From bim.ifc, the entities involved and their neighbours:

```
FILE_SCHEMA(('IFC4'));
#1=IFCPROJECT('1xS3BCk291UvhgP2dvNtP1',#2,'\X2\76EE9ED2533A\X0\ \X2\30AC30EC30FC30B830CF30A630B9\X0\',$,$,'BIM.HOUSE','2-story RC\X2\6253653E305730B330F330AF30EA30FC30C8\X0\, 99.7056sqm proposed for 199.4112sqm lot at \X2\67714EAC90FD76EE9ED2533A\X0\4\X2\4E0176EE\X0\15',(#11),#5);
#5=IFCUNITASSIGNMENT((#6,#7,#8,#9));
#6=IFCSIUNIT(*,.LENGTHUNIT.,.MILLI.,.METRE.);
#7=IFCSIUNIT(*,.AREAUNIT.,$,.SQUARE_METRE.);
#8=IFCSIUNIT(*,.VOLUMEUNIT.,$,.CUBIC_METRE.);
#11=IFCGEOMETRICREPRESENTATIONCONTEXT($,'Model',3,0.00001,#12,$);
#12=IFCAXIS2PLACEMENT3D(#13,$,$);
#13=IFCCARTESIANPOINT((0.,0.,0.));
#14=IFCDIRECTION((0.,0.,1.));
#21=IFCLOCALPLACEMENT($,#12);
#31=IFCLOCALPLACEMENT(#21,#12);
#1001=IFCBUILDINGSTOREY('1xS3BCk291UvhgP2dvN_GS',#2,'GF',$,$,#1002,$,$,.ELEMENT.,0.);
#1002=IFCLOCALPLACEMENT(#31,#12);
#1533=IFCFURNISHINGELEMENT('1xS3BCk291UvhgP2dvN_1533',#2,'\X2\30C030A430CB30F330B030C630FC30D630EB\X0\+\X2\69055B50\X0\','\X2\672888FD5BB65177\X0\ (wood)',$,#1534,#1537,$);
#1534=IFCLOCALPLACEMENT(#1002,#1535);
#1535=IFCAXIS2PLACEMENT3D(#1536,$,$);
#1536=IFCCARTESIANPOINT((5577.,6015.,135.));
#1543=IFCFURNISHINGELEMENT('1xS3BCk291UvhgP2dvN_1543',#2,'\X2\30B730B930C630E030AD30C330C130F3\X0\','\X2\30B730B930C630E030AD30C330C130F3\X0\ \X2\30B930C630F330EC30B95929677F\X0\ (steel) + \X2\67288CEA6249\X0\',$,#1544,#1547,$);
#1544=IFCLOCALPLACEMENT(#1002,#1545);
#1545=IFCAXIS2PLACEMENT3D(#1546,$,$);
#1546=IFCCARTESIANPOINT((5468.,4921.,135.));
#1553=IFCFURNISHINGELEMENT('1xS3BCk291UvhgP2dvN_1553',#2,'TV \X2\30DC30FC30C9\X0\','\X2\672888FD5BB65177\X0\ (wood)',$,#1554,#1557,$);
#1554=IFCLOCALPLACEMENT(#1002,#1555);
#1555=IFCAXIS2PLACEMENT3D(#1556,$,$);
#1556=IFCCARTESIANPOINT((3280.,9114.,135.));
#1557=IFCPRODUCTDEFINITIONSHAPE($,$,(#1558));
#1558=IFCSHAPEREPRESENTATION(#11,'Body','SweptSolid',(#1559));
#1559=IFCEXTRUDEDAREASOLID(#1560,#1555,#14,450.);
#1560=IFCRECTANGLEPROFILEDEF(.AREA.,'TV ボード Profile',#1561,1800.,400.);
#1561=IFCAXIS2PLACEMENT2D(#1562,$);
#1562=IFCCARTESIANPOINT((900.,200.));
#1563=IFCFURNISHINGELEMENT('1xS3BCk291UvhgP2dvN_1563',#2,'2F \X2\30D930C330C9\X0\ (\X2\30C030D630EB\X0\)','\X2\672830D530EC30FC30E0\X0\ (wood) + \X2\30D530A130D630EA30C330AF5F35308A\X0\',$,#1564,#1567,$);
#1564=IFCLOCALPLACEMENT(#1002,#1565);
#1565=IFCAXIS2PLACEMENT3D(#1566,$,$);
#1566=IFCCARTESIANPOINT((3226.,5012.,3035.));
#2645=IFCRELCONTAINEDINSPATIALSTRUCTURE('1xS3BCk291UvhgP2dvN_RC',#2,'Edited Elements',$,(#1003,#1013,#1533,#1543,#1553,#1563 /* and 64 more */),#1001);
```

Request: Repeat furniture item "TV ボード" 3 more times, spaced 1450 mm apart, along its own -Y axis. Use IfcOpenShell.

```python
import ifcopenshell
import ifcopenshell.api.geometry
import ifcopenshell.api.root
import ifcopenshell.util.element
import ifcopenshell.util.placement
import ifcopenshell.util.unit

model = ifcopenshell.open("bim.ifc")
unit_scale = ifcopenshell.util.unit.calculate_unit_scale(model)


def reuse_history(source, copy):
    """copy_class also copies each property set's owner history, people and application; keep the originals."""
    for rel in copy.IsDefinedBy:
        if rel.is_a("IfcRelDefinesByProperties") and (history := rel.RelatingPropertyDefinition.OwnerHistory):
            rel.RelatingPropertyDefinition.OwnerHistory = source.OwnerHistory
            ifcopenshell.util.element.remove_deep2(model, history)


source = model.by_guid("1xS3BCk291UvhgP2dvN_1553")
base = ifcopenshell.util.placement.get_local_placement(source.ObjectPlacement)
step = -base[:3, 1] * 1.45 / unit_scale

for i in range(1, 4):
    copy = ifcopenshell.api.root.copy_class(model, product=source)
    copy.Representation = ifcopenshell.util.element.copy_deep(
        model, source.Representation, exclude=["IfcGeometricRepresentationContext", "IfcRepresentationMap"]
    )
    reuse_history(source, copy)
    matrix = base.copy()
    matrix[:3, 3] += i * step
    print("added at", matrix[:3, 3].round(3) + 0.0)
    ifcopenshell.api.geometry.edit_object_placement(model, product=copy, matrix=matrix, is_si=False)

model.write("bim_edited.ifc")
```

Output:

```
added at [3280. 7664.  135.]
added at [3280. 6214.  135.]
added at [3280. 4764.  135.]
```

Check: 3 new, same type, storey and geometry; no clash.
